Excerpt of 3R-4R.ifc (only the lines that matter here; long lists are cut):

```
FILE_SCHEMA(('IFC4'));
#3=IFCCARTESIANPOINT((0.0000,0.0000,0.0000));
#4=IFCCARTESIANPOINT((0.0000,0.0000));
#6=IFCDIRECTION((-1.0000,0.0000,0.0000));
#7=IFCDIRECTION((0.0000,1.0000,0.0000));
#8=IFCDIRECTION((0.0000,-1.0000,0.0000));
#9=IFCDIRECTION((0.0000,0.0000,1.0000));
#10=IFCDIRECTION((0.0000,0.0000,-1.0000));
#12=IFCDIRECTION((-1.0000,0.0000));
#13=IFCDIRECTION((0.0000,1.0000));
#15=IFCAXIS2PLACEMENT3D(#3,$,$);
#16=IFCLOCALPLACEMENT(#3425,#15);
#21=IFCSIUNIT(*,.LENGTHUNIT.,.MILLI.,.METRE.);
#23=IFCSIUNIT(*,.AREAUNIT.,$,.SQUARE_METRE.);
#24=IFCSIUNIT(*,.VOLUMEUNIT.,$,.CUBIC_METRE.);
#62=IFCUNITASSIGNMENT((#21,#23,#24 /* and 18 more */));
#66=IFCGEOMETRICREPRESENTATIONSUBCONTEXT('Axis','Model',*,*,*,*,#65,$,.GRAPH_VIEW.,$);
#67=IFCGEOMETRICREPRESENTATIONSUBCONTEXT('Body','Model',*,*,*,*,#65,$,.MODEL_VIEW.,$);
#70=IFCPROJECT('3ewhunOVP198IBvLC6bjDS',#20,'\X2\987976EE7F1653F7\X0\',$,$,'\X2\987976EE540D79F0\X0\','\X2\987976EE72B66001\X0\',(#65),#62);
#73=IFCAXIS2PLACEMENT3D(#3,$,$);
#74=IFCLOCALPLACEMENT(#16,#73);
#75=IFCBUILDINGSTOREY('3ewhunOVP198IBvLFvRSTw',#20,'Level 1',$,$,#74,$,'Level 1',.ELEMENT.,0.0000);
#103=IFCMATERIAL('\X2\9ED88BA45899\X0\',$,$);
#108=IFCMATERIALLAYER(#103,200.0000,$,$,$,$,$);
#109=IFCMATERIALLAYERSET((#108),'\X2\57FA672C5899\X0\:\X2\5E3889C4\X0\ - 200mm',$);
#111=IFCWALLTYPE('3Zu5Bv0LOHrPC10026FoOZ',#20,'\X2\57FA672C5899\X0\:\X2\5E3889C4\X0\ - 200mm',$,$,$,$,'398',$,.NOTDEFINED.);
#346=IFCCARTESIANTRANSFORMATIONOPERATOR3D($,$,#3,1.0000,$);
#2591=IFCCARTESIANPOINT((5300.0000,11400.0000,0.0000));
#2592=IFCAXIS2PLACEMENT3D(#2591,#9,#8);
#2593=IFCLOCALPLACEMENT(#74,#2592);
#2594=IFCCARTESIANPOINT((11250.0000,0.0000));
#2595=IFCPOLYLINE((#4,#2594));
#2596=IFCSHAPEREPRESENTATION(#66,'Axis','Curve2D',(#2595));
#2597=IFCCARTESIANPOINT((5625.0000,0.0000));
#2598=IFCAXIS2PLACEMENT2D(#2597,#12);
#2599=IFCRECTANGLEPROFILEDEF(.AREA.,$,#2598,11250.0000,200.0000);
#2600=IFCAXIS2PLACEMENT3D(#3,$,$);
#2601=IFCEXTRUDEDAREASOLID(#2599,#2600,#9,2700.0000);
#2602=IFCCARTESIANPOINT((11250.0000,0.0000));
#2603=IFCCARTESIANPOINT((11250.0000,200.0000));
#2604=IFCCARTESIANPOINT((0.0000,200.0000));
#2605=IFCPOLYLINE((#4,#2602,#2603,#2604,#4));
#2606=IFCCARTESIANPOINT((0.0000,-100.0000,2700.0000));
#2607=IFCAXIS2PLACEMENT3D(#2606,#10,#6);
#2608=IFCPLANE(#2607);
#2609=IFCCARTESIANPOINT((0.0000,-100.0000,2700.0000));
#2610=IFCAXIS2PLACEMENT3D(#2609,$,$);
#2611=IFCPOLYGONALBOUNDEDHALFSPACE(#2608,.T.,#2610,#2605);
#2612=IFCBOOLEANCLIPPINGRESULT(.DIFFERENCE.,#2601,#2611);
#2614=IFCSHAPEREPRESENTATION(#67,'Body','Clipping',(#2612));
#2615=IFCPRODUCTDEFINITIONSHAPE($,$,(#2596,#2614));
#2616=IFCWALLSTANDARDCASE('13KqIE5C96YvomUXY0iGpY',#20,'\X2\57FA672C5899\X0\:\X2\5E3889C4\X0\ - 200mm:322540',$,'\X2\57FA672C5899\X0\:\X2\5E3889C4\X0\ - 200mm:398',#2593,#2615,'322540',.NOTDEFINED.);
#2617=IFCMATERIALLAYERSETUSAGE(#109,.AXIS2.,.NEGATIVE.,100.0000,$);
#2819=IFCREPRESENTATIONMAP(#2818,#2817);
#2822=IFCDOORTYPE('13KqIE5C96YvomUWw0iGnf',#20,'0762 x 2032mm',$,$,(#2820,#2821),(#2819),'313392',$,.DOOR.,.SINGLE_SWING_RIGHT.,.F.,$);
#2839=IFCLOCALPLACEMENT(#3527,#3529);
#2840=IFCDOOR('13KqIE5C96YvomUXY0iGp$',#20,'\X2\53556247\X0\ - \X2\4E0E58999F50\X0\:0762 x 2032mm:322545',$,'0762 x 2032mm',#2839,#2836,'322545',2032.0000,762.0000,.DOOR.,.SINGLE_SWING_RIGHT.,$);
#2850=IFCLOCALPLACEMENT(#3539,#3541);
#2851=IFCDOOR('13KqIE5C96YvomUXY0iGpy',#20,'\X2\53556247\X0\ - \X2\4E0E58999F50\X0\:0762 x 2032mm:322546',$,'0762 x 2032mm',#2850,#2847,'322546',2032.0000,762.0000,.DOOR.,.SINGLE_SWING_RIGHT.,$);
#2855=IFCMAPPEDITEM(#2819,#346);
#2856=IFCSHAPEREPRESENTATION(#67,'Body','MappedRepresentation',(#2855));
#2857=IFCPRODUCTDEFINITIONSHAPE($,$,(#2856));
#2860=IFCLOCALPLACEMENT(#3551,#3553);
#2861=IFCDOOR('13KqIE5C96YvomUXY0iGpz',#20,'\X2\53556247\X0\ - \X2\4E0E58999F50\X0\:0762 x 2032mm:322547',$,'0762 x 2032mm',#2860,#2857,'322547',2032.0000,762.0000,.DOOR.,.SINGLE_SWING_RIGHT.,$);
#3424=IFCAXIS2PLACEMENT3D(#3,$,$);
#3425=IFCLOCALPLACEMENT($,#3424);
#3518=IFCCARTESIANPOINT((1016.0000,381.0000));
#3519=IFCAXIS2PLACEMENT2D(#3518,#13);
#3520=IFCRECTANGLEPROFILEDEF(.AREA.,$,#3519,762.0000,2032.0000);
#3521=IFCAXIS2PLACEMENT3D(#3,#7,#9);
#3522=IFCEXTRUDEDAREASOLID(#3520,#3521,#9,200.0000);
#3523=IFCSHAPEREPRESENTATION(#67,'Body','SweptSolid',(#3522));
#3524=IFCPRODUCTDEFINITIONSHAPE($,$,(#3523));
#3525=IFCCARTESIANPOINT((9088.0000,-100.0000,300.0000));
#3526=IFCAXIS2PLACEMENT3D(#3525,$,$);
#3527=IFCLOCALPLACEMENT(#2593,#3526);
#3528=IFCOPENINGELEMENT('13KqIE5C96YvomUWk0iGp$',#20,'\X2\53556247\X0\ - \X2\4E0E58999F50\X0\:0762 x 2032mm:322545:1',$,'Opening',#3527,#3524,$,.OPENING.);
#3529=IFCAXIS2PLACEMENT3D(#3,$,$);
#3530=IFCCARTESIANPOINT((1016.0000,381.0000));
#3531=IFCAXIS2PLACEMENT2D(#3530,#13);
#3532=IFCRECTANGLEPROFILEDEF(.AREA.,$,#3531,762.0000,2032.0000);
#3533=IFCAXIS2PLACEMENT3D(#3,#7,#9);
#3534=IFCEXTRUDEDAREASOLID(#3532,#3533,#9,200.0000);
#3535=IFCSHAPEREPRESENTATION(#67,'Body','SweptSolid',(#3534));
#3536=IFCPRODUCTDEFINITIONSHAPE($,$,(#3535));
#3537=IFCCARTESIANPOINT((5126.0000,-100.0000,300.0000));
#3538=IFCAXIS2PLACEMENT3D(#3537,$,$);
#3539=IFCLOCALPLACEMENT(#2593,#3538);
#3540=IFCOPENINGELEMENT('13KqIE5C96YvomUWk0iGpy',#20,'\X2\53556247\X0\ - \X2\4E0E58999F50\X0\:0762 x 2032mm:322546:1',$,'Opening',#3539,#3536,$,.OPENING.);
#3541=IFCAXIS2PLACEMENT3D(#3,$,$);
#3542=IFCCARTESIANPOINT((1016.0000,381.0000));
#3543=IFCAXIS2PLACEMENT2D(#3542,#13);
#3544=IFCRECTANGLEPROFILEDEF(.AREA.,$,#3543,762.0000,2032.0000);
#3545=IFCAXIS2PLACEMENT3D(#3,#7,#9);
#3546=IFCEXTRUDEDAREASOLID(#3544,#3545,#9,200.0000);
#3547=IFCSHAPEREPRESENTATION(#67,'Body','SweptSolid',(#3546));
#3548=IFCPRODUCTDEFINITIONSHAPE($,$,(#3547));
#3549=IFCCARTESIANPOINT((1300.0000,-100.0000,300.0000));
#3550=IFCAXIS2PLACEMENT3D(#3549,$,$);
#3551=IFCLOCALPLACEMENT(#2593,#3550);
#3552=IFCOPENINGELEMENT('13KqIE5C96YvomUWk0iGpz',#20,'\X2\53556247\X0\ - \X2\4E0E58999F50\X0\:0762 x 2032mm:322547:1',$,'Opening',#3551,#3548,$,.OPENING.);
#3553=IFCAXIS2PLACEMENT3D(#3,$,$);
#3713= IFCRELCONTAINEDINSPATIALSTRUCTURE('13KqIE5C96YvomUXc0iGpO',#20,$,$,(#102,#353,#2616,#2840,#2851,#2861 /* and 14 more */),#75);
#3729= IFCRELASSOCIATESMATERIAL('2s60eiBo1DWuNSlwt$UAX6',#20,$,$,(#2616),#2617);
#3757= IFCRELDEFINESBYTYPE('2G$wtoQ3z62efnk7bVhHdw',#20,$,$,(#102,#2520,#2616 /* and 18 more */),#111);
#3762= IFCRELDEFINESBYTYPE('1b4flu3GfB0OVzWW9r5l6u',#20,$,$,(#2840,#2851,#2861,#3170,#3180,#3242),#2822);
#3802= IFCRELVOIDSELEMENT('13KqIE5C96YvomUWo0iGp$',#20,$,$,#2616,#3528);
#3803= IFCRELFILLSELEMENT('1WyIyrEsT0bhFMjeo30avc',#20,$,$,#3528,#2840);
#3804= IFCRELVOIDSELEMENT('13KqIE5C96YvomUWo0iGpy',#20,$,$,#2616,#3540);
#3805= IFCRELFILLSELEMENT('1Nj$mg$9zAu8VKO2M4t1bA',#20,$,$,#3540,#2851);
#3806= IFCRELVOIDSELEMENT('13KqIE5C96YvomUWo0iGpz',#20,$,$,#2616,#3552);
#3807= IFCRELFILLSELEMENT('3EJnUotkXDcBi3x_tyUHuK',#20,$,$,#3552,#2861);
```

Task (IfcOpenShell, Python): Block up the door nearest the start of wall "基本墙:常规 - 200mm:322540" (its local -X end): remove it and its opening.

```python
import ifcopenshell
import ifcopenshell.api.feature
import ifcopenshell.api.root
import ifcopenshell.geom
import ifcopenshell.util.shape

model = ifcopenshell.open("3R-4R.ifc")
settings = ifcopenshell.geom.settings()


def volume(element):
    """Net volume in cubic metres, openings subtracted."""
    shape = ifcopenshell.geom.create_shape(settings, element)
    return ifcopenshell.util.shape.get_volume(shape.geometry)


door = model.by_guid("13KqIE5C96YvomUXY0iGpz")
opening = door.FillsVoids[0].RelatingOpeningElement
wall = opening.VoidsElements[0].RelatingBuildingElement
before = volume(wall)

ifcopenshell.api.root.remove_product(model, product=door)
ifcopenshell.api.feature.remove_feature(model, feature=opening)

after = volume(wall)

print(f"wall volume {before:.3f} -> {after:.3f} m3")

model.write("3R-4R-out.ifc")
```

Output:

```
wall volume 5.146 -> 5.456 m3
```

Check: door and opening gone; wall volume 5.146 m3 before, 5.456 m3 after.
